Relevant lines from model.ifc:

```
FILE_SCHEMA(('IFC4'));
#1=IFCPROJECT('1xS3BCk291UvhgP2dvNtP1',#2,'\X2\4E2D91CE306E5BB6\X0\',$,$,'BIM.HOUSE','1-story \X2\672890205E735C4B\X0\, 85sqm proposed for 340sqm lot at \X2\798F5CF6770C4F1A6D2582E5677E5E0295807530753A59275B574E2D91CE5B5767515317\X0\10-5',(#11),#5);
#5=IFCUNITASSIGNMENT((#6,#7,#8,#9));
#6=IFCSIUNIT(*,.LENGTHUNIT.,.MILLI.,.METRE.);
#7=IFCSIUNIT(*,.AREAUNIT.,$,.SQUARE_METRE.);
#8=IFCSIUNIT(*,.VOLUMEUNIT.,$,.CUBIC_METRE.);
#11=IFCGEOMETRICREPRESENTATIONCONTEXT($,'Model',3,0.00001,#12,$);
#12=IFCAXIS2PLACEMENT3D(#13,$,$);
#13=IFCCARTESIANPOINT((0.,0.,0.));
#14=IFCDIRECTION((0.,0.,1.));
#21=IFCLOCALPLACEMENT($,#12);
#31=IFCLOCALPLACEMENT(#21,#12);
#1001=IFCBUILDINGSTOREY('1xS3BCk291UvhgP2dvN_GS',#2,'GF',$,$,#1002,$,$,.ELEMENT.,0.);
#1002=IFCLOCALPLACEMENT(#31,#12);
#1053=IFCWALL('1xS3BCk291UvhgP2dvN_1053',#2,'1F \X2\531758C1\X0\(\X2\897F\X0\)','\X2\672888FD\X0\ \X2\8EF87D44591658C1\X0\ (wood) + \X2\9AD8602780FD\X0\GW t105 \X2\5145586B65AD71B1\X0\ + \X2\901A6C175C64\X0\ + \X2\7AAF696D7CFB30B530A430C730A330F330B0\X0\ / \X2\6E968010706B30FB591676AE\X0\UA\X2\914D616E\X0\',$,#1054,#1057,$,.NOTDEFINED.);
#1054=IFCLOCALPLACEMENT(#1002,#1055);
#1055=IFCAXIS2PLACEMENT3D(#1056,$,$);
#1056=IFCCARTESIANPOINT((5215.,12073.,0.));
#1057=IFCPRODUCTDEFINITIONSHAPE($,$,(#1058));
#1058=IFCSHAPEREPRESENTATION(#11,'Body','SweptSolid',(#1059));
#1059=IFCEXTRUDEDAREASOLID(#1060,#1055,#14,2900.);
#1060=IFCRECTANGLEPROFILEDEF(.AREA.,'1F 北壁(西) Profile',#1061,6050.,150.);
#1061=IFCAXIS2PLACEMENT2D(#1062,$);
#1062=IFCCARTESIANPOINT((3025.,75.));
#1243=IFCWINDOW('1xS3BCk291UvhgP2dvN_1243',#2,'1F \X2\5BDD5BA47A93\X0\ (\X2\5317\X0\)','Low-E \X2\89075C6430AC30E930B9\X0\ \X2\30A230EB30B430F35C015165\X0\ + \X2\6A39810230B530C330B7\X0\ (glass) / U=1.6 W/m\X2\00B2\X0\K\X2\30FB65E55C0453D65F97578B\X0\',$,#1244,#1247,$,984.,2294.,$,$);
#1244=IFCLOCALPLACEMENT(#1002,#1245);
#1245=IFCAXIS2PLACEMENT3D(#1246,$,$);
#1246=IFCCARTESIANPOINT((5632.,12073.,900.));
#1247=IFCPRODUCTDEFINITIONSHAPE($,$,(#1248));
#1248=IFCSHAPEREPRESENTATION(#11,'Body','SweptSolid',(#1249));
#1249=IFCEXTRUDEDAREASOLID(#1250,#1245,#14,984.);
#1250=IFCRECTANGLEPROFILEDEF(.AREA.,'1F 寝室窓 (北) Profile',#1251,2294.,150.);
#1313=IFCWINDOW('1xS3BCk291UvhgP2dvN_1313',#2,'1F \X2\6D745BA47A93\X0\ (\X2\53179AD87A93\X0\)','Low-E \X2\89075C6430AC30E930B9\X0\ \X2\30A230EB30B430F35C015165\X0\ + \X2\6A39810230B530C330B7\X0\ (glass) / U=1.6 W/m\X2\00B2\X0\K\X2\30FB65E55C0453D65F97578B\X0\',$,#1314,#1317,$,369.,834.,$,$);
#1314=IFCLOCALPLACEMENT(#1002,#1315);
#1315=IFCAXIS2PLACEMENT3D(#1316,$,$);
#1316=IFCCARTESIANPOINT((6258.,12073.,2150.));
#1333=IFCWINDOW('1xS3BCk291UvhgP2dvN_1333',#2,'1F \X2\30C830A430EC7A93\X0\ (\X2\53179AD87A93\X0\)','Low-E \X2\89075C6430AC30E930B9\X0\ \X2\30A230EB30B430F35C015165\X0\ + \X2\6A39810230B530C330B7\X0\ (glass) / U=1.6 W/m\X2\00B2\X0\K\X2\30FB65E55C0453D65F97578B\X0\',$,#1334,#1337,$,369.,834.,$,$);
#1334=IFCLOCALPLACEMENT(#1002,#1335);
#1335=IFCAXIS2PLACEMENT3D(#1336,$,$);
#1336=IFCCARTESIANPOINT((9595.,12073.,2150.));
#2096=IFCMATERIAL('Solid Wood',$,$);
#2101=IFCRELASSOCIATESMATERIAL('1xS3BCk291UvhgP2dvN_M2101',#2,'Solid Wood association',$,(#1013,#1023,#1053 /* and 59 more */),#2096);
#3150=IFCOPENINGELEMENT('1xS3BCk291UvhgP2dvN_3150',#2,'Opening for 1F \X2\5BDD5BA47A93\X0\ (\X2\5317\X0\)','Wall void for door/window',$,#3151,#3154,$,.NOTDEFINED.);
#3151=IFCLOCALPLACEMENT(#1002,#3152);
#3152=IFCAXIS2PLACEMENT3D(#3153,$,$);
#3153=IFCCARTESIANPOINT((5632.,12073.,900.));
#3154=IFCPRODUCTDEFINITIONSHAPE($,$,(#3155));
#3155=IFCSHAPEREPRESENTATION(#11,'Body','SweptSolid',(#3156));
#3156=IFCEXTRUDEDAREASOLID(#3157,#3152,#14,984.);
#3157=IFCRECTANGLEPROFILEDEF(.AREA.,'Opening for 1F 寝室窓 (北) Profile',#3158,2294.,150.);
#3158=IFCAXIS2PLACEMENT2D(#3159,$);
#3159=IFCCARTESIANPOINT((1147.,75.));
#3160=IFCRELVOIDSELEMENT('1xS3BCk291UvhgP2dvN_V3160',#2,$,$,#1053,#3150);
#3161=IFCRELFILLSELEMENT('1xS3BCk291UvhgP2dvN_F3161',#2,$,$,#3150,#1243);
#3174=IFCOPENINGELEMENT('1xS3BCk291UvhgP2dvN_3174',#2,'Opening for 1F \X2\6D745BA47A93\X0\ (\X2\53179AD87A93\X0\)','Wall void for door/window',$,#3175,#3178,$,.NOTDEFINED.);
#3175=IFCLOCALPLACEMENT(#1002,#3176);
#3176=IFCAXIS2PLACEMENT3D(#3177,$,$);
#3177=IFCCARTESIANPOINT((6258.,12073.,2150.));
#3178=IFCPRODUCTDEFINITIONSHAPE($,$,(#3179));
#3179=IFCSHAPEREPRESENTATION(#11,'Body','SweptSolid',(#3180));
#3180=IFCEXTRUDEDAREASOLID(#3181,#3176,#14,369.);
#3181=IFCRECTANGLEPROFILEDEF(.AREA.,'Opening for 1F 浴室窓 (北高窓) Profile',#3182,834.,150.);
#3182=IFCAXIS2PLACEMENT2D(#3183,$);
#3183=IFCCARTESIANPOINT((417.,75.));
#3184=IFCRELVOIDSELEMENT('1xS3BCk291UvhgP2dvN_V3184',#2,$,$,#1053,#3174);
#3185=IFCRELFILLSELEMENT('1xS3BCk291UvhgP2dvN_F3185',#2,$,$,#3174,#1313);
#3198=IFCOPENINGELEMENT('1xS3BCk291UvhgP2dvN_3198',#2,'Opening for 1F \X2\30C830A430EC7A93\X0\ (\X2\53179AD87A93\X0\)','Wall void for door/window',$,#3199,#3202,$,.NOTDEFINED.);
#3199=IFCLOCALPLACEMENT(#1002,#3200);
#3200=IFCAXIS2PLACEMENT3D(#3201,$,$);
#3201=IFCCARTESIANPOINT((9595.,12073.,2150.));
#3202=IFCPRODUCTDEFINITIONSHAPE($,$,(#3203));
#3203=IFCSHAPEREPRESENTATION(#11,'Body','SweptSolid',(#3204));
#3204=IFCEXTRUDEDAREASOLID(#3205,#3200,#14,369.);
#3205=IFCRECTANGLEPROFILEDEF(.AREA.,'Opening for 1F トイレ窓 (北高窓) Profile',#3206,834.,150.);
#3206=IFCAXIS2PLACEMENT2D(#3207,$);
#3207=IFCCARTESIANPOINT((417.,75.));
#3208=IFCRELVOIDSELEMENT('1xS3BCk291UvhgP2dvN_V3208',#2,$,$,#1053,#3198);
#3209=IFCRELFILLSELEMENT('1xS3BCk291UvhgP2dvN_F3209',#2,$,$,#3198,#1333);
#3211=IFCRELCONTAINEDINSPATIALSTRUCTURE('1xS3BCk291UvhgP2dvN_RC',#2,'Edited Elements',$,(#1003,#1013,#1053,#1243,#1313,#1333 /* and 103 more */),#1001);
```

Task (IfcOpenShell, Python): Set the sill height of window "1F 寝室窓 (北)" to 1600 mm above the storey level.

```python
import numpy as np
import ifcopenshell
import ifcopenshell.api.geometry
import ifcopenshell.geom
import ifcopenshell.util.element
import ifcopenshell.util.placement
import ifcopenshell.util.shape
import ifcopenshell.util.unit

model = ifcopenshell.open("model.ifc")
unit_scale = ifcopenshell.util.unit.calculate_unit_scale(model)

window = model.by_id(1243)
opening = window.FillsVoids[0].RelatingOpeningElement
storey = ifcopenshell.util.element.get_container(window, ifc_class="IfcBuildingStorey")
level = ifcopenshell.util.placement.get_local_placement(storey.ObjectPlacement)[2, 3]

# The opening's origin need not be at the sill, so measure its lowest point.
shape = ifcopenshell.geom.create_shape(ifcopenshell.geom.settings(), opening)
bottom = ifcopenshell.util.shape.get_shape_bottom_elevation(shape, shape.geometry) / unit_scale
dz = level + 1600.0 - bottom

shift = np.array([0.0, 0.0, dz])
# The window is not placed relative to its opening, so move both.
for product in (opening, window):
    matrix = ifcopenshell.util.placement.get_local_placement(product.ObjectPlacement)
    matrix[:3, 3] += shift
    ifcopenshell.api.geometry.edit_object_placement(model, product=product, matrix=matrix, is_si=False)

print(f"moved by {dz * unit_scale:+.3f} m")

model.write("model_v2.ifc")
```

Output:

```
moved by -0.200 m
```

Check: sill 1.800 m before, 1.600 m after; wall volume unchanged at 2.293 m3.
